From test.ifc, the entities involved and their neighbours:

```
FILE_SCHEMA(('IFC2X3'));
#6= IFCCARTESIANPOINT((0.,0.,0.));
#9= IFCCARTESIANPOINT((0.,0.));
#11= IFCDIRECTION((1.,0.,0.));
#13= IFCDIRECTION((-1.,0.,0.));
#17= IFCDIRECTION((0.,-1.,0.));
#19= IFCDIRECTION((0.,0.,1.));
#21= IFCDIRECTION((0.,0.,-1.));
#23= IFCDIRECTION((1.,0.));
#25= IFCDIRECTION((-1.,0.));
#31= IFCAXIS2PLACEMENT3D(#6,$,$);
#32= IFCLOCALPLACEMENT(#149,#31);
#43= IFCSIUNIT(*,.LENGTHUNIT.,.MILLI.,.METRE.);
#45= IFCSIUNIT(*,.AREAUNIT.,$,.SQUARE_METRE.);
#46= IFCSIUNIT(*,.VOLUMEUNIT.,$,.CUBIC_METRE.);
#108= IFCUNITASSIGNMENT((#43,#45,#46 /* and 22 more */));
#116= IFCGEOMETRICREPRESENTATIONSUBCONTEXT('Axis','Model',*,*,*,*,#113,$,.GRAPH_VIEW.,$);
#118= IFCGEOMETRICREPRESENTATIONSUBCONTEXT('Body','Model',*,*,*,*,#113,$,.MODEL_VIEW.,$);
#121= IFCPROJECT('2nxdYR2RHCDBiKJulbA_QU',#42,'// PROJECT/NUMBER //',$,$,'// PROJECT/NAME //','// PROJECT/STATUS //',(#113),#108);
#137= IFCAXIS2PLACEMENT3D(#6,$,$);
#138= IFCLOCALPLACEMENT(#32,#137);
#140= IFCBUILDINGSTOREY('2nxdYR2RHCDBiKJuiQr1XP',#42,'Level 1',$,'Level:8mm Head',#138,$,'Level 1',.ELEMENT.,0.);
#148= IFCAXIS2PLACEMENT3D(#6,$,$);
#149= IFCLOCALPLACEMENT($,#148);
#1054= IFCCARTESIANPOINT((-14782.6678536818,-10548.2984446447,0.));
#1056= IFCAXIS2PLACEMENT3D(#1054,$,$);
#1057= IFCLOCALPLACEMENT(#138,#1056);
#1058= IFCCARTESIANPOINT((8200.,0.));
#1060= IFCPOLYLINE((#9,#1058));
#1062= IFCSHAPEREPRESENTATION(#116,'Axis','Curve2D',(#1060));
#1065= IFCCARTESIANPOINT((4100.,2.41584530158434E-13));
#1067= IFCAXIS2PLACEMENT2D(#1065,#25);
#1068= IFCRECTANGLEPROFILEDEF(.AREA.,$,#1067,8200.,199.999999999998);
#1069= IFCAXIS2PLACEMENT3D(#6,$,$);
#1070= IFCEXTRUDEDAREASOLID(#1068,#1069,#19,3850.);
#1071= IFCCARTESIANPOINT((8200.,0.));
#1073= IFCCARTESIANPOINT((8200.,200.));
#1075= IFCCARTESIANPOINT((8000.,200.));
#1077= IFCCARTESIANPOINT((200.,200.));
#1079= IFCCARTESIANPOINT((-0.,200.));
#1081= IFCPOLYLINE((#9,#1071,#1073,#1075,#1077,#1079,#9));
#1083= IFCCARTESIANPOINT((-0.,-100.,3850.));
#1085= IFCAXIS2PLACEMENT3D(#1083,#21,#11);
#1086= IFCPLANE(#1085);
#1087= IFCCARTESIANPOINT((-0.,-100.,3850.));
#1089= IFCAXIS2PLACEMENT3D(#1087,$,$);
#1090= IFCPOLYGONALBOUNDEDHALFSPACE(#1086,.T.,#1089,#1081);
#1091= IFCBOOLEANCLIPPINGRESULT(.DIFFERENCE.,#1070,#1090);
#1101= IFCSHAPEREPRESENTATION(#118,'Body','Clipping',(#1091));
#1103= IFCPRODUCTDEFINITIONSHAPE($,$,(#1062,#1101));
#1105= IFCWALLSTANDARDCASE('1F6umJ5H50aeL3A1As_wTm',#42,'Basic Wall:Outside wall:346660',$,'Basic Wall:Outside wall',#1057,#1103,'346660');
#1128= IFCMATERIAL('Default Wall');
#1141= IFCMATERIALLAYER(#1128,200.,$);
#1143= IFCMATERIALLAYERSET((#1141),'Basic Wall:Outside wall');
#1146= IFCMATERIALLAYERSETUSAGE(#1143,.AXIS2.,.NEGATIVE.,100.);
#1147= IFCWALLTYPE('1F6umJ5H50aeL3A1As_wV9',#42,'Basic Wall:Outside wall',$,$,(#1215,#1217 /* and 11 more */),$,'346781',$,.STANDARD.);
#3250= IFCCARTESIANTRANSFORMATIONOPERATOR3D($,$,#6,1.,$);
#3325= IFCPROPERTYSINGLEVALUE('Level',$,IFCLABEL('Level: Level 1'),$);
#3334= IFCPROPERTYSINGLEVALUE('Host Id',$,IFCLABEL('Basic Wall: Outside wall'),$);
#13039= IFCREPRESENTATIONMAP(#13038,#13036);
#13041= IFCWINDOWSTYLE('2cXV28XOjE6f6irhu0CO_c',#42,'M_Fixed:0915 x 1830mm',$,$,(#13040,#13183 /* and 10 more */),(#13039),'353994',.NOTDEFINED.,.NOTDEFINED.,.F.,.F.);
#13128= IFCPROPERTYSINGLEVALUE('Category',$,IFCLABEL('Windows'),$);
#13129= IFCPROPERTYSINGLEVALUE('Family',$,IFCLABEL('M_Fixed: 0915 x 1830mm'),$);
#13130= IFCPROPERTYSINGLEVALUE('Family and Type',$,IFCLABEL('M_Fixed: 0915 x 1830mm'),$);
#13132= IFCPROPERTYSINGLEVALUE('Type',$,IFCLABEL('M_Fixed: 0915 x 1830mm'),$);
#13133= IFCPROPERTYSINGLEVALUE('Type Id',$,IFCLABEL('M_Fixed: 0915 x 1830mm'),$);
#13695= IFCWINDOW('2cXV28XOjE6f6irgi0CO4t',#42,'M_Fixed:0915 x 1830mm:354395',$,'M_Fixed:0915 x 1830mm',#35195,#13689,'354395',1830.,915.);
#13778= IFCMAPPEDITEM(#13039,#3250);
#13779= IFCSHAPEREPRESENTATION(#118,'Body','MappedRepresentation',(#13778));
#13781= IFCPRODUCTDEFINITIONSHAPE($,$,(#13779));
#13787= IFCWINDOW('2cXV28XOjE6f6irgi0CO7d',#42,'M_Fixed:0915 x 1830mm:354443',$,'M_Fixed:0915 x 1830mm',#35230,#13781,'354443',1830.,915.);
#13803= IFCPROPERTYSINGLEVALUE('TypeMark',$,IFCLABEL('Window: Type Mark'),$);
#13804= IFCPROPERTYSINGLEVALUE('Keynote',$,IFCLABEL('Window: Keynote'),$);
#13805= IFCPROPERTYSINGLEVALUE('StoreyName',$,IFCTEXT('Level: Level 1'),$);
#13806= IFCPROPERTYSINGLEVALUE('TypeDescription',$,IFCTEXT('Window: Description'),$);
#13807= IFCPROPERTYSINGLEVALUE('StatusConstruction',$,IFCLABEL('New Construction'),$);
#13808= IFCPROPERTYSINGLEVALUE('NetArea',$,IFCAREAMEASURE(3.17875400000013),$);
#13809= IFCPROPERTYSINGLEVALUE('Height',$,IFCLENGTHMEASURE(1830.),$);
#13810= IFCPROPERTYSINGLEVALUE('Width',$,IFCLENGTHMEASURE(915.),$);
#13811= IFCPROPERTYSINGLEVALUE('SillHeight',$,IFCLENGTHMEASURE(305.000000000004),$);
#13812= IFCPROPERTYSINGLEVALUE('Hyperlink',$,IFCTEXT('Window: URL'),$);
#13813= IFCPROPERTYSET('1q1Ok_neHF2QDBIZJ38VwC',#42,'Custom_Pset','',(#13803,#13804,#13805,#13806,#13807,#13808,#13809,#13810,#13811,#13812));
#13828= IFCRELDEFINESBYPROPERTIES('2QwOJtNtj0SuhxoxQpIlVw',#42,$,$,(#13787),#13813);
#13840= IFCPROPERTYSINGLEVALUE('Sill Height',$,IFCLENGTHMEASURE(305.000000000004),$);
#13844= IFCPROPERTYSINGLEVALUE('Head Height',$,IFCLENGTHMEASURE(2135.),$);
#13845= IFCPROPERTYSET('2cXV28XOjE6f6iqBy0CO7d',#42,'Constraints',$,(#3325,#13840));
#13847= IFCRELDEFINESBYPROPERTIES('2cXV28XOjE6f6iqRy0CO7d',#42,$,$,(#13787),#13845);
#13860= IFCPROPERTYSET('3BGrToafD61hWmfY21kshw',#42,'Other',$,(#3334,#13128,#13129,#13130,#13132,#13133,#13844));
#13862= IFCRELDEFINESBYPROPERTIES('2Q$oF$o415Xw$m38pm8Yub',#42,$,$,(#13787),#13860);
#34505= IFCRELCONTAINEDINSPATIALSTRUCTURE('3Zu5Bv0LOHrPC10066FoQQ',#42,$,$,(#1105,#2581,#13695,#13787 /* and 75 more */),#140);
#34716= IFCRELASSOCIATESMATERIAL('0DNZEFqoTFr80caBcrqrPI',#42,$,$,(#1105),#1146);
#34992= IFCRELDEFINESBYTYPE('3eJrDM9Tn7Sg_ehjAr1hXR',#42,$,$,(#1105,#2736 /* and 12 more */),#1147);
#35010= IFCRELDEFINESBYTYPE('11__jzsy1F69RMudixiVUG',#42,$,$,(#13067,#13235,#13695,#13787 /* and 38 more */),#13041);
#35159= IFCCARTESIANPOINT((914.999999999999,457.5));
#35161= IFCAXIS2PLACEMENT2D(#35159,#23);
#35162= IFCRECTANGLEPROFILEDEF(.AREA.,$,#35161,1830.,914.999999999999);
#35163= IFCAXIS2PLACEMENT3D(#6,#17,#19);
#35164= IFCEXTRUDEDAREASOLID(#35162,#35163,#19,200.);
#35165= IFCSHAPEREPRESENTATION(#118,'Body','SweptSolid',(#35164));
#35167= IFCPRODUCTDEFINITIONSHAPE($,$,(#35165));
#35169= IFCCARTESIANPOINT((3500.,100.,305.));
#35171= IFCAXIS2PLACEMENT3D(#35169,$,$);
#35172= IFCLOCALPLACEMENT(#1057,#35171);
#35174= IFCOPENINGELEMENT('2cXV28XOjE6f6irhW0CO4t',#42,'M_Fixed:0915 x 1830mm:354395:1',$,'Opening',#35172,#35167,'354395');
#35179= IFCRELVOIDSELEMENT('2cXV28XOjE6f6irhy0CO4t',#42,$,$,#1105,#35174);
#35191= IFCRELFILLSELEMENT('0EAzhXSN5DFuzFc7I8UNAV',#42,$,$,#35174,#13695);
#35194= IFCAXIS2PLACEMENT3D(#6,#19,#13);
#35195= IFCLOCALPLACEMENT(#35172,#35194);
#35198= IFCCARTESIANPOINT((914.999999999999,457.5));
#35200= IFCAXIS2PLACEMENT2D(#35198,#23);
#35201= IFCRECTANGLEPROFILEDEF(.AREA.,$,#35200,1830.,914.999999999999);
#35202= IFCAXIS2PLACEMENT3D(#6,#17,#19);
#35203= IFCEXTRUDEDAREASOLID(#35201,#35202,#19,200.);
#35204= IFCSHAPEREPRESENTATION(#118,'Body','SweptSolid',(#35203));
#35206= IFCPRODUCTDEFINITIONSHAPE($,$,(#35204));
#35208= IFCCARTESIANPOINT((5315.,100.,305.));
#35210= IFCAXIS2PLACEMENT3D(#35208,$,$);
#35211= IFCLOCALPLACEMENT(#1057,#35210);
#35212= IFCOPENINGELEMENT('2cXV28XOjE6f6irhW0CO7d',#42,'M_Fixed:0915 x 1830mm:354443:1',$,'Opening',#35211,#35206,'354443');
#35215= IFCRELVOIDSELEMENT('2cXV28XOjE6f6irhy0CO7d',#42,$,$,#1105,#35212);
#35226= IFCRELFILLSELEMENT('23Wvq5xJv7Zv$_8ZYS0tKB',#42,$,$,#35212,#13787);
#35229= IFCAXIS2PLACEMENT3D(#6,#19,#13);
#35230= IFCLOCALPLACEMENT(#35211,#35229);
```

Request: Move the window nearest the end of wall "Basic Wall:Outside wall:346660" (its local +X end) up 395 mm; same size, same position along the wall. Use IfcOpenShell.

```python
import numpy as np
import ifcopenshell
import ifcopenshell.api.geometry
import ifcopenshell.api.pset
import ifcopenshell.util.element
import ifcopenshell.util.placement
import ifcopenshell.util.unit

model = ifcopenshell.open("test.ifc")
unit_scale = ifcopenshell.util.unit.calculate_unit_scale(model)

window = model.by_id(13787)
opening = window.FillsVoids[0].RelatingOpeningElement
dz = 0.395 / unit_scale

shift = np.array([0.0, 0.0, dz])
# The window is placed relative to its opening, so it follows when the opening moves.
matrix = ifcopenshell.util.placement.get_local_placement(opening.ObjectPlacement)
matrix[:3, 3] += shift
ifcopenshell.api.geometry.edit_object_placement(
    model, product=opening, matrix=matrix, is_si=False, should_transform_children=True
)

# Keep the stored heights in step.
pset = model.by_id(ifcopenshell.util.element.get_pset(window, "Custom_Pset", should_inherit=False)["id"])
ifcopenshell.api.pset.edit_pset(model, pset=pset, properties={
    "SillHeight": model.create_entity("IfcLengthMeasure", ifcopenshell.util.element.get_pset(window, "Constraints", "Sill Height") + dz),
})
pset = model.by_id(ifcopenshell.util.element.get_pset(window, "Constraints", should_inherit=False)["id"])
ifcopenshell.api.pset.edit_pset(model, pset=pset, properties={
    "Sill Height": model.create_entity("IfcLengthMeasure", ifcopenshell.util.element.get_pset(window, "Constraints", "Sill Height") + dz),
})
pset = model.by_id(ifcopenshell.util.element.get_pset(window, "Other", should_inherit=False)["id"])
ifcopenshell.api.pset.edit_pset(model, pset=pset, properties={
    "Head Height": model.create_entity("IfcLengthMeasure", ifcopenshell.util.element.get_pset(window, "Other", "Head Height") + dz),
})

print(f"moved by {dz * unit_scale:+.3f} m")

model.write("test-out.ifc")
```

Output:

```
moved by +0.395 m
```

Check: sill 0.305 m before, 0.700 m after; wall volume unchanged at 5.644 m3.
